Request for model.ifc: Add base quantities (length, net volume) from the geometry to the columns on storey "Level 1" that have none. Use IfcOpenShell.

First a look at what the model holds.

```python
import ifcopenshell
import ifcopenshell.util.element
import ifcopenshell.util.unit

model = ifcopenshell.open("model.ifc")
print(model.schema)
for unit_type in ("LENGTHUNIT", "AREAUNIT", "VOLUMEUNIT"):
    print(unit_type, ifcopenshell.util.unit.calculate_unit_scale(model, unit_type))
storey = next(s for s in model.by_type("IfcBuildingStorey") if s.Name == "Level 1")
columns = [e for e in ifcopenshell.util.element.get_decomposition(storey) if e.is_a("IfcColumn")]
for e in sorted(columns, key=lambda e: e.id()):
    print(e.id(), e.is_a(), e.Name, list(ifcopenshell.util.element.get_psets(e, qtos_only=True)), sep=" | ")
```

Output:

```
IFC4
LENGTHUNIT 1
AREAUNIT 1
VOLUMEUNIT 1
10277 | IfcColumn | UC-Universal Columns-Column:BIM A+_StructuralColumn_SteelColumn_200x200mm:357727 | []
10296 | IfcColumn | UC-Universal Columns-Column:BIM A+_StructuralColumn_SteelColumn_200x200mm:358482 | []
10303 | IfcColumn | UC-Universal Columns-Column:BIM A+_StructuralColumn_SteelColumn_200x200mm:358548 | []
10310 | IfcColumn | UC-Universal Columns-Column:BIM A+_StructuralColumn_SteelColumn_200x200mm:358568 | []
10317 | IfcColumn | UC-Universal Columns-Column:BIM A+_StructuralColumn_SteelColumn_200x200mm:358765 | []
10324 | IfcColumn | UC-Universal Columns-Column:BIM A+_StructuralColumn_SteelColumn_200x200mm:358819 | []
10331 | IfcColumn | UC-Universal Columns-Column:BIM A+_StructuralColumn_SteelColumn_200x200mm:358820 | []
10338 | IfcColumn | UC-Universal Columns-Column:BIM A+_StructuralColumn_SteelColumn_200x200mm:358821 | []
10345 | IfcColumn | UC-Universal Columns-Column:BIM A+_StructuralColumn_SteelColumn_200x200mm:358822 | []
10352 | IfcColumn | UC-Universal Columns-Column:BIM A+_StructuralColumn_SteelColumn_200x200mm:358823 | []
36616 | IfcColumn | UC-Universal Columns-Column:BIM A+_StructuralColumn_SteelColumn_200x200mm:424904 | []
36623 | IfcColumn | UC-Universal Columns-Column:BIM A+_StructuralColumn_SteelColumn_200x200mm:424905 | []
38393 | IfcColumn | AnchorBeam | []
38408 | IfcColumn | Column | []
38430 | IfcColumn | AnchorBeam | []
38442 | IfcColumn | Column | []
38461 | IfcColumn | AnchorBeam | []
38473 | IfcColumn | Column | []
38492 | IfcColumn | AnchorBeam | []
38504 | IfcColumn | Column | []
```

```python
import ifcopenshell
import ifcopenshell.api.pset
import ifcopenshell.geom
import ifcopenshell.util.element
import ifcopenshell.util.shape
import ifcopenshell.util.unit

model = ifcopenshell.open("model.ifc")
unit_scale = ifcopenshell.util.unit.calculate_unit_scale(model)
volume_scale = ifcopenshell.util.unit.calculate_unit_scale(model, "VOLUMEUNIT")
settings = ifcopenshell.geom.settings()

storey = next(s for s in model.by_type("IfcBuildingStorey") if s.Name == "Level 1")
columns = [e for e in ifcopenshell.util.element.get_decomposition(storey) if e.is_a("IfcColumn")]

for e in sorted(columns, key=lambda e: e.id()):
    if ifcopenshell.util.element.get_psets(e, qtos_only=True, should_inherit=False):
        continue
    # Geometry comes back in metres, in the element's own axes.
    shape = ifcopenshell.geom.create_shape(settings, e)
    values = {
        "Length": ifcopenshell.util.shape.get_z(shape.geometry) / unit_scale,
        "NetVolume": ifcopenshell.util.shape.get_volume(shape.geometry) / volume_scale,
    }
    qto = ifcopenshell.api.pset.add_qto(model, product=e, name="Qto_ColumnBaseQuantities")
    ifcopenshell.api.pset.edit_qto(model, qto=qto, properties=values)
    print(e.id(), {k: round(v, 3) for k, v in values.items()})

model.write("model_rev.ifc")
```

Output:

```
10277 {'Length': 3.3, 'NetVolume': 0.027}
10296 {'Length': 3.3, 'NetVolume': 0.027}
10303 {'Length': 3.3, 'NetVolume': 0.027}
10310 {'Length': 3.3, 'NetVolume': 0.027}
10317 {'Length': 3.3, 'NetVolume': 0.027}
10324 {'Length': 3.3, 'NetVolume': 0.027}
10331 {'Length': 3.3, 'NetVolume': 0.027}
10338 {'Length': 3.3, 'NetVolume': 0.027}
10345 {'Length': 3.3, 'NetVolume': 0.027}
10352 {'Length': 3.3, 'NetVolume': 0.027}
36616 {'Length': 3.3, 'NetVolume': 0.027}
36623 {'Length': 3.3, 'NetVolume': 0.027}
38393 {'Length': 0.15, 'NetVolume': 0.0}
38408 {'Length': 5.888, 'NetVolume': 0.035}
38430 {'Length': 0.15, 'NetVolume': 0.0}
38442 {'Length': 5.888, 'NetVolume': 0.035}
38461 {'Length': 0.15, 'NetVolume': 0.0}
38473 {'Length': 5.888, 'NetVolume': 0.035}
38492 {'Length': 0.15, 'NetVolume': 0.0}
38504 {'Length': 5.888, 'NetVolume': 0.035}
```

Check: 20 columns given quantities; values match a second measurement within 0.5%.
